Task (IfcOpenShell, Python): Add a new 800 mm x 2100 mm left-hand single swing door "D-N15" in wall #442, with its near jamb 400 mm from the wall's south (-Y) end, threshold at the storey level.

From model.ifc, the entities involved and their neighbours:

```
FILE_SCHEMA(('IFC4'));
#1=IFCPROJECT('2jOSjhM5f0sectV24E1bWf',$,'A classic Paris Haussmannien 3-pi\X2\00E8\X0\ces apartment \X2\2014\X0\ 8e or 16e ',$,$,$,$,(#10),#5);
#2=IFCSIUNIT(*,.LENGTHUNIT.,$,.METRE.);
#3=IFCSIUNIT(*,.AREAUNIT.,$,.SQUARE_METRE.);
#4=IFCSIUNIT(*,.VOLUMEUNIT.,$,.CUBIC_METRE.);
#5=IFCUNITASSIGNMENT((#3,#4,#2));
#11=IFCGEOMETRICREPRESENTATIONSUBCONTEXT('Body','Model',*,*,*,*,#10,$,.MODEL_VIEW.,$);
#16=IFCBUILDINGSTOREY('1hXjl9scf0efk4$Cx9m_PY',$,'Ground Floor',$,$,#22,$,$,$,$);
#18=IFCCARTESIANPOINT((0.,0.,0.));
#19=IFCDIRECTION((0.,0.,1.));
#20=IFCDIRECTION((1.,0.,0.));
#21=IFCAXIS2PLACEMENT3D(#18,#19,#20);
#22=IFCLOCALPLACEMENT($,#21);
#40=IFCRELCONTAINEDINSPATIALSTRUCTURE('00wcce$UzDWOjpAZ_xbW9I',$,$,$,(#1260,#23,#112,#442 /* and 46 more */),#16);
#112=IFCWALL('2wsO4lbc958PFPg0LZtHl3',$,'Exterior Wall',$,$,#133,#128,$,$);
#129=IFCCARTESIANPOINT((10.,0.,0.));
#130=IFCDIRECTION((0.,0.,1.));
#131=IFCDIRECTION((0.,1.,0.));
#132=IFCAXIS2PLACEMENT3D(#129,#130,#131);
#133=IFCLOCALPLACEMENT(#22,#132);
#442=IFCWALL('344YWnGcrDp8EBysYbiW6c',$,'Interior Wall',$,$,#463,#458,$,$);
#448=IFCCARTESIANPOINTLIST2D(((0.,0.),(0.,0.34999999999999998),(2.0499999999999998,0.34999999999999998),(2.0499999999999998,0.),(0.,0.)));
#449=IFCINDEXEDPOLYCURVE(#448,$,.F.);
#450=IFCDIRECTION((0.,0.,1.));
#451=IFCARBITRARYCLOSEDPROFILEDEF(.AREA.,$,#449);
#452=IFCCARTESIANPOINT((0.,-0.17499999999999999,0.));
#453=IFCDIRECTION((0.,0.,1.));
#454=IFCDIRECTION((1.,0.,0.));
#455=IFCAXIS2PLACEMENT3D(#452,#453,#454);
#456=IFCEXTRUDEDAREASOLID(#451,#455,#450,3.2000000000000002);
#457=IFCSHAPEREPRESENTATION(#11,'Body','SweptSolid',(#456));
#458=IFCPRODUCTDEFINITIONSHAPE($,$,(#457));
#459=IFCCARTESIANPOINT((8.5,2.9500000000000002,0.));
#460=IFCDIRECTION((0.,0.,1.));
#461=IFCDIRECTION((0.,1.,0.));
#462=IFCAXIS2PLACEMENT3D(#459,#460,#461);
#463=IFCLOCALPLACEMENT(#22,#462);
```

```python
import numpy as np
import ifcopenshell
import ifcopenshell.api.feature
import ifcopenshell.api.geometry
import ifcopenshell.api.root
import ifcopenshell.api.spatial
import ifcopenshell.geom
import ifcopenshell.util.element
import ifcopenshell.util.placement
import ifcopenshell.util.representation
import ifcopenshell.util.shape
import ifcopenshell.util.unit

model = ifcopenshell.open("model.ifc")
unit_scale = ifcopenshell.util.unit.calculate_unit_scale(model)
settings = ifcopenshell.geom.settings()


def volume(element):
    """Net volume in cubic metres, openings subtracted."""
    shape = ifcopenshell.geom.create_shape(settings, element)
    return ifcopenshell.util.shape.get_volume(shape.geometry)


wall = model.by_guid("344YWnGcrDp8EBysYbiW6c")
storey = ifcopenshell.util.element.get_container(wall, ifc_class="IfcBuildingStorey")
context = ifcopenshell.util.representation.get_context(model, "Model", "Body", "MODEL_VIEW")
before = volume(wall)

width, height, from_end, sill = 0.8, 2.1, 0.4, 0.0  # metres

# The wall runs along its own X axis, and the end named is its -X end.
wall_shape = ifcopenshell.geom.create_shape(settings, wall)
x, y, z = ifcopenshell.util.shape.get_vertices(wall_shape.geometry).T
start = x.min() + from_end
face, thickness = float(y.min()), float(y.max() - y.min())
wall_matrix = ifcopenshell.util.placement.get_local_placement(wall.ObjectPlacement)
level = ifcopenshell.util.placement.get_local_placement(storey.ObjectPlacement)[2, 3]


def in_wall(x, y):
    """Placement at x, y metres in the wall's axes, at sill height."""
    matrix = wall_matrix.copy()
    matrix[:, 3] = wall_matrix @ np.array([x / unit_scale, y / unit_scale, 0.0, 1.0])
    matrix[2, 3] = level + sill / unit_scale
    return matrix


# Opening: a box that overshoots both wall faces by 50 mm.
opening = ifcopenshell.api.root.create_entity(model, ifc_class="IfcOpeningElement", predefined_type="OPENING")
box = ifcopenshell.api.geometry.add_wall_representation(
    model, context=context, length=width, height=height, thickness=thickness + 0.1
)
ifcopenshell.api.geometry.assign_representation(model, product=opening, representation=box)
ifcopenshell.api.geometry.edit_object_placement(model, product=opening, matrix=in_wall(start, face - 0.05), is_si=False)
ifcopenshell.api.feature.add_feature(model, feature=opening, element=wall)

door = ifcopenshell.api.root.create_entity(model, ifc_class="IfcDoor", name="D-N15", predefined_type="DOOR")
door.OverallWidth, door.OverallHeight = width / unit_scale, height / unit_scale
door.OperationType = "SINGLE_SWING_LEFT"
body = ifcopenshell.api.geometry.add_door_representation(
    model,
    context=context,
    overall_width=door.OverallWidth,
    overall_height=door.OverallHeight,
    operation_type="SINGLE_SWING_LEFT",
    lining_properties={"LiningDepth": thickness / unit_scale, "ThresholdDepth": thickness / unit_scale},
)
ifcopenshell.api.geometry.assign_representation(model, product=door, representation=body)
ifcopenshell.api.spatial.assign_container(model, products=[door], relating_structure=storey)
ifcopenshell.api.feature.add_filling(model, opening=opening, element=door)

# The lining spans the wall, so the door starts at the wall face.
ifcopenshell.api.geometry.edit_object_placement(model, product=door, matrix=in_wall(start, face), is_si=False)

after = volume(wall)

print(f"wall volume {before:.3f} -> {after:.3f} m3")

model.write("model_edited.ifc")
```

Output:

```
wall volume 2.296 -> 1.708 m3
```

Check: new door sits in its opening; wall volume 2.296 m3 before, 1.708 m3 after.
